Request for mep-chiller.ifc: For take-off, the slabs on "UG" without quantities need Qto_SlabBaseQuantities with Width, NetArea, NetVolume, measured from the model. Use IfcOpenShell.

First a look at what the model holds.

```python
import ifcopenshell
import ifcopenshell.util.element
import ifcopenshell.util.unit

model = ifcopenshell.open("mep-chiller.ifc")
print(model.schema)
for unit_type in ("LENGTHUNIT", "AREAUNIT", "VOLUMEUNIT"):
    print(unit_type, ifcopenshell.util.unit.calculate_unit_scale(model, unit_type))
storey = next(s for s in model.by_type("IfcBuildingStorey") if s.Name == "UG")
slabs = [e for e in ifcopenshell.util.element.get_decomposition(storey) if e.is_a("IfcSlab")]
for e in sorted(slabs, key=lambda e: e.id()):
    print(e.id(), e.is_a(), e.Name, list(ifcopenshell.util.element.get_psets(e, qtos_only=True)), sep=" | ")
```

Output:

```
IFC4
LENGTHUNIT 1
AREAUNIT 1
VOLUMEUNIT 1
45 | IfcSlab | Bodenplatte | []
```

```python
import ifcopenshell
import ifcopenshell.api.pset
import ifcopenshell.geom
import ifcopenshell.util.element
import ifcopenshell.util.shape
import ifcopenshell.util.unit

model = ifcopenshell.open("mep-chiller.ifc")
unit_scale = ifcopenshell.util.unit.calculate_unit_scale(model)
area_scale = ifcopenshell.util.unit.calculate_unit_scale(model, "AREAUNIT")
volume_scale = ifcopenshell.util.unit.calculate_unit_scale(model, "VOLUMEUNIT")
settings = ifcopenshell.geom.settings()

storey = next(s for s in model.by_type("IfcBuildingStorey") if s.Name == "UG")
slabs = [e for e in ifcopenshell.util.element.get_decomposition(storey) if e.is_a("IfcSlab")]

for e in sorted(slabs, key=lambda e: e.id()):
    if ifcopenshell.util.element.get_psets(e, qtos_only=True, should_inherit=False):
        continue
    # Geometry comes back in metres, in the element's own axes.
    shape = ifcopenshell.geom.create_shape(settings, e)
    values = {
        "Width": ifcopenshell.util.shape.get_z(shape.geometry) / unit_scale,
        "NetArea": ifcopenshell.util.shape.get_footprint_area(shape.geometry) / area_scale,
        "NetVolume": ifcopenshell.util.shape.get_volume(shape.geometry) / volume_scale,
    }
    qto = ifcopenshell.api.pset.add_qto(model, product=e, name="Qto_SlabBaseQuantities")
    ifcopenshell.api.pset.edit_qto(model, qto=qto, properties=values)
    print(e.id(), {k: round(v, 3) for k, v in values.items()})

model.write("mep-chiller_edited.ifc")
```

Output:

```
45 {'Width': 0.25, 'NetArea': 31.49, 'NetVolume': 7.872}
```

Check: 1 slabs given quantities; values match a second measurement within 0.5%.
